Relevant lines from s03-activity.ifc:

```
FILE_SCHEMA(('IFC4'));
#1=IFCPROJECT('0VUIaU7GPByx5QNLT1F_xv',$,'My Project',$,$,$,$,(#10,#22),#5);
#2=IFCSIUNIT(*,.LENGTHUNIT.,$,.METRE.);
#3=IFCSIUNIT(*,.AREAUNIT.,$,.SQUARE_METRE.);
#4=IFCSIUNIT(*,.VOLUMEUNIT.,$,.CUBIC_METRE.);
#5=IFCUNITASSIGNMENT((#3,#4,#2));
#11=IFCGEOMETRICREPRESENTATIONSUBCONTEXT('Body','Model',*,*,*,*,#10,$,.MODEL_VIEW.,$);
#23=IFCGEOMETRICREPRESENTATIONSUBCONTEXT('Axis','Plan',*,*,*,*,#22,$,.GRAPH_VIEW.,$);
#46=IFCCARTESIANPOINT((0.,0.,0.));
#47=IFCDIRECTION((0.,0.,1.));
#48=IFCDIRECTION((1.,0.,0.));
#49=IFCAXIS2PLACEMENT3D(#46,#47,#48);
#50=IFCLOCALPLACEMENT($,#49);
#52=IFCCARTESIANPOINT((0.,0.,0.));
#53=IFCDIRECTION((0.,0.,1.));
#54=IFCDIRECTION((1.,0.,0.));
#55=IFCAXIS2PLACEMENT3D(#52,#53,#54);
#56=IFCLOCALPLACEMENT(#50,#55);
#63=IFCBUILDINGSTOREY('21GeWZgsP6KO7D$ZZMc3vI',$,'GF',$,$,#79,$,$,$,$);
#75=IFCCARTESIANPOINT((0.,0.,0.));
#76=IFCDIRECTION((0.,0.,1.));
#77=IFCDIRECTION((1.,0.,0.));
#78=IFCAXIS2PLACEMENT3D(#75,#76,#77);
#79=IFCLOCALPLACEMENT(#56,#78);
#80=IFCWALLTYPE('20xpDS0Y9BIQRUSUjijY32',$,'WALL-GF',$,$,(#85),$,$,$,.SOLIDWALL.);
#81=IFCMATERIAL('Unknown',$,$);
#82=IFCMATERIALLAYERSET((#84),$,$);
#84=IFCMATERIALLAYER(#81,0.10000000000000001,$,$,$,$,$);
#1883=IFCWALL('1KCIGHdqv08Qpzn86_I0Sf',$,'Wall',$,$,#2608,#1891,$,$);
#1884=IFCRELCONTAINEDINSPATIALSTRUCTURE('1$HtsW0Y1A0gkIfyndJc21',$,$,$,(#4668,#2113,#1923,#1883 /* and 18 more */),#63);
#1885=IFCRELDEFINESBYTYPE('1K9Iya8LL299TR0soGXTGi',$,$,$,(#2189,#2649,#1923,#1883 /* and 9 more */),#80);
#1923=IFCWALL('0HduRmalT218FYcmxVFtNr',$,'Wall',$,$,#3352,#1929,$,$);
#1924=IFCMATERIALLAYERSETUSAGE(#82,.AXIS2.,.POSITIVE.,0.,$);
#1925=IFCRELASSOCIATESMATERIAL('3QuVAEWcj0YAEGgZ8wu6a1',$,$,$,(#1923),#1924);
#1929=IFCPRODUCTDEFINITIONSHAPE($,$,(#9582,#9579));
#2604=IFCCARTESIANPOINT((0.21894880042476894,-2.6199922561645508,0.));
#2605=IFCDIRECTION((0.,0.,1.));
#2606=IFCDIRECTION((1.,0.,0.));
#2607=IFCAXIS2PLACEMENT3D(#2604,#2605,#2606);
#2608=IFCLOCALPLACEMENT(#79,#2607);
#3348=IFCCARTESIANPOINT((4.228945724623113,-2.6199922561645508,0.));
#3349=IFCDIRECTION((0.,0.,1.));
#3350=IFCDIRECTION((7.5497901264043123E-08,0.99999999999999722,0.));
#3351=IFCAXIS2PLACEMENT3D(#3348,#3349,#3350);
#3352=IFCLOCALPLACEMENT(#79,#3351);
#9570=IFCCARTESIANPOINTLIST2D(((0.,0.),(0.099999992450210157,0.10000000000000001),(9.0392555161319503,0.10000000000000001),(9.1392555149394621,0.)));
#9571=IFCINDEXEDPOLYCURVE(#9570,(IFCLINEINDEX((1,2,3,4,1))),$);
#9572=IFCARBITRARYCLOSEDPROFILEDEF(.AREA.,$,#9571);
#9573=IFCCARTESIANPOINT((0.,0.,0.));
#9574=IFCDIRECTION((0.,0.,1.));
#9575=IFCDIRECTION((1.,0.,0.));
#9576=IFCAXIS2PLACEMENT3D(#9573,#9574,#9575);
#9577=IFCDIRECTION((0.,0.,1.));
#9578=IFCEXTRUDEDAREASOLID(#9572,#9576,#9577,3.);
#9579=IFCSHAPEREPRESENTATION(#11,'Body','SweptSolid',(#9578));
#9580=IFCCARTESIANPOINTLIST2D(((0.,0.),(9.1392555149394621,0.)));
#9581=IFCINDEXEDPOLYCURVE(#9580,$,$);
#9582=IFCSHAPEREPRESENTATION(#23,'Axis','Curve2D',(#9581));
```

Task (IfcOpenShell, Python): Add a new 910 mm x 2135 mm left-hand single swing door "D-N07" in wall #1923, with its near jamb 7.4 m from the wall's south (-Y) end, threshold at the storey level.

```python
import numpy as np
import ifcopenshell
import ifcopenshell.api.feature
import ifcopenshell.api.geometry
import ifcopenshell.api.root
import ifcopenshell.api.spatial
import ifcopenshell.geom
import ifcopenshell.util.element
import ifcopenshell.util.placement
import ifcopenshell.util.representation
import ifcopenshell.util.shape
import ifcopenshell.util.unit

model = ifcopenshell.open("s03-activity.ifc")
unit_scale = ifcopenshell.util.unit.calculate_unit_scale(model)
settings = ifcopenshell.geom.settings()


def volume(element):
    """Net volume in cubic metres, openings subtracted."""
    shape = ifcopenshell.geom.create_shape(settings, element)
    return ifcopenshell.util.shape.get_volume(shape.geometry)


wall = model.by_guid("0HduRmalT218FYcmxVFtNr")
storey = ifcopenshell.util.element.get_container(wall, ifc_class="IfcBuildingStorey")
context = ifcopenshell.util.representation.get_context(model, "Model", "Body", "MODEL_VIEW")
before = volume(wall)

width, height, from_end, sill = 0.91, 2.135, 7.4, 0.0  # metres

# The wall runs along its own X axis, and the end named is its -X end.
wall_shape = ifcopenshell.geom.create_shape(settings, wall)
x, y, z = ifcopenshell.util.shape.get_vertices(wall_shape.geometry).T
start = x.min() + from_end
face, thickness = float(y.min()), float(y.max() - y.min())
wall_matrix = ifcopenshell.util.placement.get_local_placement(wall.ObjectPlacement)
level = ifcopenshell.util.placement.get_local_placement(storey.ObjectPlacement)[2, 3]


def in_wall(x, y):
    """Placement at x, y metres in the wall's axes, at sill height."""
    matrix = wall_matrix.copy()
    matrix[:, 3] = wall_matrix @ np.array([x / unit_scale, y / unit_scale, 0.0, 1.0])
    matrix[2, 3] = level + sill / unit_scale
    return matrix


# Opening: a box that overshoots both wall faces by 50 mm.
opening = ifcopenshell.api.root.create_entity(model, ifc_class="IfcOpeningElement", predefined_type="OPENING")
box = ifcopenshell.api.geometry.add_wall_representation(
    model, context=context, length=width, height=height, thickness=thickness + 0.1
)
ifcopenshell.api.geometry.assign_representation(model, product=opening, representation=box)
ifcopenshell.api.geometry.edit_object_placement(model, product=opening, matrix=in_wall(start, face - 0.05), is_si=False)
ifcopenshell.api.feature.add_feature(model, feature=opening, element=wall)

door = ifcopenshell.api.root.create_entity(model, ifc_class="IfcDoor", name="D-N07", predefined_type="DOOR")
door.OverallWidth, door.OverallHeight = width / unit_scale, height / unit_scale
door.OperationType = "SINGLE_SWING_LEFT"
body = ifcopenshell.api.geometry.add_door_representation(
    model,
    context=context,
    overall_width=door.OverallWidth,
    overall_height=door.OverallHeight,
    operation_type="SINGLE_SWING_LEFT",
    lining_properties={"LiningDepth": thickness / unit_scale, "ThresholdDepth": thickness / unit_scale},
)
ifcopenshell.api.geometry.assign_representation(model, product=door, representation=body)
ifcopenshell.api.spatial.assign_container(model, products=[door], relating_structure=storey)
ifcopenshell.api.feature.add_filling(model, opening=opening, element=door)

# The lining spans the wall, so the door starts at the wall face.
ifcopenshell.api.geometry.edit_object_placement(model, product=door, matrix=in_wall(start, face), is_si=False)

after = volume(wall)

print(f"wall volume {before:.3f} -> {after:.3f} m3")

model.write("s03-activity-out.ifc")
```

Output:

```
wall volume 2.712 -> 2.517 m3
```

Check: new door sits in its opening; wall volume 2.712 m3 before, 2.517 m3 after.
